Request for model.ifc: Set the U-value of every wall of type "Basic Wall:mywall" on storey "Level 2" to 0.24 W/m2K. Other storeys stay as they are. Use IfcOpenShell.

First a look at what the model holds.

```python
import ifcopenshell
import ifcopenshell.util.element

model = ifcopenshell.open("model.ifc")
print(model.schema)
storey = next(s for s in model.by_type("IfcBuildingStorey") if s.Name == "Level 2")
walls = [e for e in ifcopenshell.util.element.get_decomposition(storey) if e.is_a("IfcWall")]
seen = {}
for e in walls:
    element_type = ifcopenshell.util.element.get_type(e)
    key = (element_type.Name if element_type != e and element_type else None, ifcopenshell.util.element.get_pset(e, "Pset_WallCommon", "ThermalTransmittance"))
    seen[key] = seen.get(key, 0) + 1
for (name, value), count in sorted(seen.items(), key=str):
    print(count, "x", name, "|", value)
```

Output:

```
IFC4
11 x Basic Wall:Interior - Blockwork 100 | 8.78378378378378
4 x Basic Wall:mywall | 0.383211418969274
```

```python
import ifcopenshell
import ifcopenshell.api.pset
import ifcopenshell.util.element

model = ifcopenshell.open("model.ifc")

storey = next(s for s in model.by_type("IfcBuildingStorey") if s.Name == "Level 2")
walls = [e for e in ifcopenshell.util.element.get_decomposition(storey) if e.is_a("IfcWall")]

count = 0
for e in walls:
    element_type = ifcopenshell.util.element.get_type(e)
    if element_type in (None, e) or element_type.Name != "Basic Wall:mywall":
        continue
    # add_pset returns the element's existing set when there is one.
    pset = ifcopenshell.api.pset.add_pset(model, product=e, name="Pset_WallCommon")
    ifcopenshell.api.pset.edit_pset(model, pset=pset, properties={"ThermalTransmittance": 0.24})
    count += 1

print(count, "walls updated")

model.write("model_rev.ifc")
```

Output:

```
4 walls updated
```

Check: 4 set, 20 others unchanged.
